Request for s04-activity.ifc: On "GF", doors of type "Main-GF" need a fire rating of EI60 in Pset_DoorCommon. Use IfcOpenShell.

First a look at what the model holds.

```python
import ifcopenshell
import ifcopenshell.util.element

model = ifcopenshell.open("s04-activity.ifc")
print(model.schema)
storey = next(s for s in model.by_type("IfcBuildingStorey") if s.Name == "GF")
doors = [e for e in ifcopenshell.util.element.get_decomposition(storey) if e.is_a("IfcDoor")]
seen = {}
for e in doors:
    element_type = ifcopenshell.util.element.get_type(e)
    key = (element_type.Name if element_type != e and element_type else None, ifcopenshell.util.element.get_pset(e, "Pset_DoorCommon", "FireRating"))
    seen[key] = seen.get(key, 0) + 1
for (name, value), count in sorted(seen.items(), key=str):
    print(count, "x", name, "|", value)
```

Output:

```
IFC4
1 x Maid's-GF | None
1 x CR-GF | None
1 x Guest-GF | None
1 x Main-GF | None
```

```python
import ifcopenshell
import ifcopenshell.api.pset
import ifcopenshell.util.element

model = ifcopenshell.open("s04-activity.ifc")

storey = next(s for s in model.by_type("IfcBuildingStorey") if s.Name == "GF")
doors = [e for e in ifcopenshell.util.element.get_decomposition(storey) if e.is_a("IfcDoor")]

count = 0
for e in doors:
    element_type = ifcopenshell.util.element.get_type(e)
    if element_type in (None, e) or element_type.Name != "Main-GF":
        continue
    # add_pset returns the element's existing set when there is one.
    pset = ifcopenshell.api.pset.add_pset(model, product=e, name="Pset_DoorCommon")
    ifcopenshell.api.pset.edit_pset(model, pset=pset, properties={"FireRating": "EI60"})
    count += 1

print(count, "doors updated")

model.write("s04-activity_updated.ifc")
```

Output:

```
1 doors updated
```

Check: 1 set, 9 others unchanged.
